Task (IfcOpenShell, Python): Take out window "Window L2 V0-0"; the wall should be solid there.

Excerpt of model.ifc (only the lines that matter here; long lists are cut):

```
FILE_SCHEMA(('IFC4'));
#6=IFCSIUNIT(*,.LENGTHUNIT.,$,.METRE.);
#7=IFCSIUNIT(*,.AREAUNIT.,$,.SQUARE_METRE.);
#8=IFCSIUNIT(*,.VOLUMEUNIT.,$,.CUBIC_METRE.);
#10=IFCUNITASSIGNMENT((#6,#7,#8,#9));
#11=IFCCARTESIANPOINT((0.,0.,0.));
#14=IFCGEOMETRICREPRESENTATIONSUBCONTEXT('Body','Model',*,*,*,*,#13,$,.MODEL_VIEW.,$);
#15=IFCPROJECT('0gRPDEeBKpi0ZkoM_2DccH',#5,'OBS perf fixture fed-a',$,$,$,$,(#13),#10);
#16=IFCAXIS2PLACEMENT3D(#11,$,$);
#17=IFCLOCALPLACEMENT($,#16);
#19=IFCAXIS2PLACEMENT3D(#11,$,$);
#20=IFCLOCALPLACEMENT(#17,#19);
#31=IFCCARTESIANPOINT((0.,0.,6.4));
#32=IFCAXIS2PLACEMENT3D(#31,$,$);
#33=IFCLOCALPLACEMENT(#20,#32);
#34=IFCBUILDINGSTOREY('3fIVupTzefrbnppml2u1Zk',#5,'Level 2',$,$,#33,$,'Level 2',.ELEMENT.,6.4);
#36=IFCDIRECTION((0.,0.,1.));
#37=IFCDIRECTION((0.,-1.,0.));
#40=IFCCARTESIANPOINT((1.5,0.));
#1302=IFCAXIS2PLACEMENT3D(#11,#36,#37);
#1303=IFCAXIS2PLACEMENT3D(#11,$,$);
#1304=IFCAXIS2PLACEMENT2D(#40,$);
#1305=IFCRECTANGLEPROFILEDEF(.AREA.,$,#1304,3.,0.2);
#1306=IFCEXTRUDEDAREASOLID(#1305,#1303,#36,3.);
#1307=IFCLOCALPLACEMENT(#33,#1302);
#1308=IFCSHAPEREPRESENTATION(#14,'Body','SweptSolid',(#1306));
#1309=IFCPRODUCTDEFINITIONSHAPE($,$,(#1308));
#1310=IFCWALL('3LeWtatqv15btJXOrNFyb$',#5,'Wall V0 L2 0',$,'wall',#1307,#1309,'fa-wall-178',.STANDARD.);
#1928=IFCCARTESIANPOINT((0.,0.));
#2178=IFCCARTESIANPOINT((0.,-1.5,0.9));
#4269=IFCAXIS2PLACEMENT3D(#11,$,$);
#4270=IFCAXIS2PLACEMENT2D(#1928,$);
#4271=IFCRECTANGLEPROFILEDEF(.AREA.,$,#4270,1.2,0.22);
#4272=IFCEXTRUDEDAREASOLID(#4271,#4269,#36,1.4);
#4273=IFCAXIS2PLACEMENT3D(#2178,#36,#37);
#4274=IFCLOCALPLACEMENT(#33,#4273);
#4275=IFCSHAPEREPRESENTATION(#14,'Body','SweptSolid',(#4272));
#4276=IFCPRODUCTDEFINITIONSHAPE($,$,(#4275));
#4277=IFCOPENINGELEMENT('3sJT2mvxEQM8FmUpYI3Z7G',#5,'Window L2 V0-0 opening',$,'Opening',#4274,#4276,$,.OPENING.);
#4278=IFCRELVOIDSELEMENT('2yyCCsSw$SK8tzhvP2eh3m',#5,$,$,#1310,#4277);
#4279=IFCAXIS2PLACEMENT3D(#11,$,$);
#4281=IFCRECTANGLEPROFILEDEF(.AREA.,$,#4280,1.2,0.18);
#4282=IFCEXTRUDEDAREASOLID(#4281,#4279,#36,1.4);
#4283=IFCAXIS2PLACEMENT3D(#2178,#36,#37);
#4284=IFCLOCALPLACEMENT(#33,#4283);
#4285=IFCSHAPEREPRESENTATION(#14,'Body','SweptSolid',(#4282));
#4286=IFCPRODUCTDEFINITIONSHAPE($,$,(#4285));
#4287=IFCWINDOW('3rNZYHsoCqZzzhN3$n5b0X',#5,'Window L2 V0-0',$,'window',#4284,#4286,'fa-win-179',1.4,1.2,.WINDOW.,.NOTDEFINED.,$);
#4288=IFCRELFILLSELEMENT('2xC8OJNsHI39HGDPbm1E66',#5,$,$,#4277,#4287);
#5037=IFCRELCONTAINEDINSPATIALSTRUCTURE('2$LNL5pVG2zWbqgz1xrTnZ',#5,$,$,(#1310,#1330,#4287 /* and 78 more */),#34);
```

```python
import ifcopenshell
import ifcopenshell.api.feature
import ifcopenshell.api.root
import ifcopenshell.geom
import ifcopenshell.util.shape

model = ifcopenshell.open("model.ifc")
settings = ifcopenshell.geom.settings()


def volume(element):
    """Net volume in cubic metres, openings subtracted."""
    shape = ifcopenshell.geom.create_shape(settings, element)
    return ifcopenshell.util.shape.get_volume(shape.geometry)


window = model.by_guid("3rNZYHsoCqZzzhN3$n5b0X")
opening = window.FillsVoids[0].RelatingOpeningElement
wall = opening.VoidsElements[0].RelatingBuildingElement
before = volume(wall)

ifcopenshell.api.root.remove_product(model, product=window)
ifcopenshell.api.feature.remove_feature(model, feature=opening)

after = volume(wall)

print(f"wall volume {before:.3f} -> {after:.3f} m3")

model.write("model_updated.ifc")
```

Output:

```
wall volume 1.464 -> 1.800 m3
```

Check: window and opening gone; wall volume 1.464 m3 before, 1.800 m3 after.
